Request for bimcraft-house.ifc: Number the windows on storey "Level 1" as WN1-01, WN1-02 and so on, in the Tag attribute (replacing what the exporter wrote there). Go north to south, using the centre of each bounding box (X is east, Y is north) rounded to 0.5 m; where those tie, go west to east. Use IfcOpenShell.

First a look at what the model holds.

```python
import ifcopenshell
import ifcopenshell.util.element
import ifcopenshell.util.placement

model = ifcopenshell.open("bimcraft-house.ifc")
print(model.schema)
storey = next(s for s in model.by_type("IfcBuildingStorey") if s.Name == "Level 1")
windows = [e for e in ifcopenshell.util.element.get_decomposition(storey) if e.is_a("IfcWindow")]
for e in sorted(windows, key=lambda e: e.id()):
    origin = ifcopenshell.util.placement.get_local_placement(e.ObjectPlacement)[:3, 3]
    print(e.id(), e.Tag, e.Name, origin.round(2) + 0.0, sep=" | ")
```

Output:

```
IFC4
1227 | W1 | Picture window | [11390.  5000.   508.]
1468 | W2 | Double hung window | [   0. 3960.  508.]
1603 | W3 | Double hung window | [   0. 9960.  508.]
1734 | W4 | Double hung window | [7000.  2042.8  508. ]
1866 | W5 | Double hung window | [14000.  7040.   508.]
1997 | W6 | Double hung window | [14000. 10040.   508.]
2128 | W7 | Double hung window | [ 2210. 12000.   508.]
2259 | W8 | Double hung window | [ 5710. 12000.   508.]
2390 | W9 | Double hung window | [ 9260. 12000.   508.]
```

```python
import ifcopenshell
import ifcopenshell.geom
import ifcopenshell.util.element
import ifcopenshell.util.shape

model = ifcopenshell.open("bimcraft-house.ifc")
settings = ifcopenshell.geom.settings()
settings.set("use-world-coords", True)


def centre(element):
    shape = ifcopenshell.geom.create_shape(settings, element)
    return ifcopenshell.util.shape.get_bbox_centroid(shape.geometry)


storey = next(s for s in model.by_type("IfcBuildingStorey") if s.Name == "Level 1")
windows = [e for e in ifcopenshell.util.element.get_decomposition(storey) if e.is_a("IfcWindow")]

# Insertion points can sit at a corner or the storey origin, so sort by the geometry (in metres).
centres = {e: centre(e) for e in windows}
windows.sort(key=lambda e: (-round(centres[e][1] / 0.5), centres[e][0]))

for i, e in enumerate(windows, start=1):
    number = f"WN1-{i:02d}"
    e.Tag = number
    print(e.id(), number)

model.write("bimcraft-house_rev.ifc")
```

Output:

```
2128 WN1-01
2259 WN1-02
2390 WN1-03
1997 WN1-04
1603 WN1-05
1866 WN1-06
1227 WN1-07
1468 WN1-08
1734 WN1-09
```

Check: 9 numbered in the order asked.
